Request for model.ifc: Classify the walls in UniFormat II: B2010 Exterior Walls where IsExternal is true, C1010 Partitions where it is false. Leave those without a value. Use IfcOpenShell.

First a look at what the model holds.

```python
import ifcopenshell
import ifcopenshell.util.element

model = ifcopenshell.open("model.ifc")
print(model.schema)
print("classifications:", [c.Name for c in model.by_type("IfcClassification")])
values = [ifcopenshell.util.element.get_pset(e, "Pset_WallCommon", "IsExternal") for e in model.by_type("IfcWall")]
for value in (True, False, None):
    print("IsExternal", value, values.count(value))
```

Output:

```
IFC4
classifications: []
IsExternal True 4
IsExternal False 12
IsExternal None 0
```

```python
import ifcopenshell
import ifcopenshell.api.classification
import ifcopenshell.util.element

model = ifcopenshell.open("model.ifc")

system = ifcopenshell.api.classification.add_classification(model, classification="UniFormat II")

walls = model.by_type("IfcWall")
external = {e: ifcopenshell.util.element.get_pset(e, "Pset_WallCommon", "IsExternal") for e in walls}
for flag, code, name in ((True, "B2010", "Exterior Walls"), (False, "C1010", "Partitions")):
    products = [e for e in walls if external[e] is flag]
    ifcopenshell.api.classification.add_reference(
        model, products=products, classification=system, identification=code, name=name
    )
    print(code, len(products))

model.write("model-out.ifc")
```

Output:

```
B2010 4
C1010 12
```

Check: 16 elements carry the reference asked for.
